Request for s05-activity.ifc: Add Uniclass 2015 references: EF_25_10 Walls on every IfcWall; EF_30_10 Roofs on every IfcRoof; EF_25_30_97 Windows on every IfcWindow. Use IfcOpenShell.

First a look at what the model holds.

```python
import ifcopenshell

model = ifcopenshell.open("s05-activity.ifc")
print(model.schema)
print("classifications:", [c.Name for c in model.by_type("IfcClassification")])
for ifc_class in ("IfcDoor", "IfcRoof", "IfcStair", "IfcWall", "IfcWindow"):
    print(ifc_class, len(model.by_type(ifc_class)))
```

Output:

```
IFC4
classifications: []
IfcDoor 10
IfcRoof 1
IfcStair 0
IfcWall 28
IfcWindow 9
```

```python
import ifcopenshell
import ifcopenshell.api.classification

model = ifcopenshell.open("s05-activity.ifc")

system = ifcopenshell.api.classification.add_classification(model, classification="Uniclass 2015")

codes = {
    "IfcWall": ("EF_25_10", "Walls"),
    "IfcRoof": ("EF_30_10", "Roofs"),
    "IfcWindow": ("EF_25_30_97", "Windows"),
}
for ifc_class, (code, name) in codes.items():
    products = model.by_type(ifc_class)
    ifcopenshell.api.classification.add_reference(
        model, products=products, classification=system, identification=code, name=name
    )
    print(code, len(products))

model.write("s05-activity_edited.ifc")
```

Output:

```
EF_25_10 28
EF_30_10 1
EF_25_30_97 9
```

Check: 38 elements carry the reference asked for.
